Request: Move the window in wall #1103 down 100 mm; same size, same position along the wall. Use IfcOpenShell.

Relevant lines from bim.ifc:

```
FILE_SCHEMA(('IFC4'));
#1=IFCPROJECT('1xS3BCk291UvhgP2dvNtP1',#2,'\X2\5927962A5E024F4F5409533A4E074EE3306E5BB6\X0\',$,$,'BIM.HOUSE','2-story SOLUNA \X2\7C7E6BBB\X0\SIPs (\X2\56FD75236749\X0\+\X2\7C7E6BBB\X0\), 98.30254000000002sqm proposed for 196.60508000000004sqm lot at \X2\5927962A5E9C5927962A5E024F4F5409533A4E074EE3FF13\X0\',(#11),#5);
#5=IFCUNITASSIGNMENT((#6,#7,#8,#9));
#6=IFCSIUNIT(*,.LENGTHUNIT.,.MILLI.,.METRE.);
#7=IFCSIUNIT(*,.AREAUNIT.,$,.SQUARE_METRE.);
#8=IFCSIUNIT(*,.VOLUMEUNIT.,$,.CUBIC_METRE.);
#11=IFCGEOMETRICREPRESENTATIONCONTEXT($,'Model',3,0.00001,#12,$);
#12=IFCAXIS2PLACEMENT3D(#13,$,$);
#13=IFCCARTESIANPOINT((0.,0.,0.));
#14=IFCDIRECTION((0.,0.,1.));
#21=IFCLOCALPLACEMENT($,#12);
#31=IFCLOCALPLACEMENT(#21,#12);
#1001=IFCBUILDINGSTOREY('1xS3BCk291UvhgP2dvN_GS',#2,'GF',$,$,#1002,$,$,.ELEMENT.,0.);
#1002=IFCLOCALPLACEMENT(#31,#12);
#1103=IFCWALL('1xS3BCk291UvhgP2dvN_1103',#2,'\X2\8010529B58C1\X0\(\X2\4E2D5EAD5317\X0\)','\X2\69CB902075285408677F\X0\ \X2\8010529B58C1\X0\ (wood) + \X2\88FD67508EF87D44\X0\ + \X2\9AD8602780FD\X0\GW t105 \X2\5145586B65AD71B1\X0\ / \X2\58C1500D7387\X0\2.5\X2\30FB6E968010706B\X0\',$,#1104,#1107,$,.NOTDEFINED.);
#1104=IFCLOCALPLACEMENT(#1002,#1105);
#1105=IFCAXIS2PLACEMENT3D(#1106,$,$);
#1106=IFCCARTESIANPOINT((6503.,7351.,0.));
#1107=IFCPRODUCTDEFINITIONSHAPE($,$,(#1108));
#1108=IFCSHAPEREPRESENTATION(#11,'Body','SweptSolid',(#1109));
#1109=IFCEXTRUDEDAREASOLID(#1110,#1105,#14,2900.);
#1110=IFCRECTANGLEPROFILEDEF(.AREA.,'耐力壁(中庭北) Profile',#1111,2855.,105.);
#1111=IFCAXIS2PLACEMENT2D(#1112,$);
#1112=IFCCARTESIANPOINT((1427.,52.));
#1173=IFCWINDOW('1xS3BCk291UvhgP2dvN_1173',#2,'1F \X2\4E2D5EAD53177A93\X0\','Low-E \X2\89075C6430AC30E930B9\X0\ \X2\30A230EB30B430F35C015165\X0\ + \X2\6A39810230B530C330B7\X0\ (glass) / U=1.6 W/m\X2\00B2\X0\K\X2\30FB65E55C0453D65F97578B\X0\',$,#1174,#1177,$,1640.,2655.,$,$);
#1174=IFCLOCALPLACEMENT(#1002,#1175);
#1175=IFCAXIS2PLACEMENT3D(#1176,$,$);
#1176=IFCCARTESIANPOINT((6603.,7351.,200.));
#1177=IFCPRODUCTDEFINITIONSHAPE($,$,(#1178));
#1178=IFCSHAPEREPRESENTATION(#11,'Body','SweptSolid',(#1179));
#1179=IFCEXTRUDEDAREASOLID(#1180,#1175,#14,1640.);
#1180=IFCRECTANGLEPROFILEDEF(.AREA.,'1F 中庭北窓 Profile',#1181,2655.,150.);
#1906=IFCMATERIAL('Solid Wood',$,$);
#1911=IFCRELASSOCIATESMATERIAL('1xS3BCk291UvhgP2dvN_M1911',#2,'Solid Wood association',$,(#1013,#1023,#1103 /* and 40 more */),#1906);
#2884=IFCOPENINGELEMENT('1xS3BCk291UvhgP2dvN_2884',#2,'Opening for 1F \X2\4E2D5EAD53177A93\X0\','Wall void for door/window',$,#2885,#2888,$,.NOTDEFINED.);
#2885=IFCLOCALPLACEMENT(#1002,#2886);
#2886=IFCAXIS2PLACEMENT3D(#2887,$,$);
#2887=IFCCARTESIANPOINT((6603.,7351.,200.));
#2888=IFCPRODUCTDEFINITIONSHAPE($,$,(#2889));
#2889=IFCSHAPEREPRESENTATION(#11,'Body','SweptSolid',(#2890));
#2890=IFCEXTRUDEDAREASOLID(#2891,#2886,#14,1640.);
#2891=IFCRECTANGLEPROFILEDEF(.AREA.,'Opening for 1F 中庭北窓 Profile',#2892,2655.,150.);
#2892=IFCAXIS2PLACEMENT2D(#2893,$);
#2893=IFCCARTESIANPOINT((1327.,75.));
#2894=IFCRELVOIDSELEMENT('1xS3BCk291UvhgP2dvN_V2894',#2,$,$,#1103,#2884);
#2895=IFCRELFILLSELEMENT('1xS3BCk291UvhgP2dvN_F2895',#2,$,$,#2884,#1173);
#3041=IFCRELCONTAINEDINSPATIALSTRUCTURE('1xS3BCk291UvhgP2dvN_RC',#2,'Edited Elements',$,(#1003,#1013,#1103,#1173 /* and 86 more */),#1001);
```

```python
import numpy as np
import ifcopenshell
import ifcopenshell.api.geometry
import ifcopenshell.util.placement
import ifcopenshell.util.unit

model = ifcopenshell.open("bim.ifc")
unit_scale = ifcopenshell.util.unit.calculate_unit_scale(model)

window = model.by_guid("1xS3BCk291UvhgP2dvN_1173")
opening = window.FillsVoids[0].RelatingOpeningElement
dz = -100.0

shift = np.array([0.0, 0.0, dz])
# The window is not placed relative to its opening, so move both.
for product in (opening, window):
    matrix = ifcopenshell.util.placement.get_local_placement(product.ObjectPlacement)
    matrix[:3, 3] += shift
    ifcopenshell.api.geometry.edit_object_placement(model, product=product, matrix=matrix, is_si=False)

print(f"moved by {dz * unit_scale:+.3f} m")

model.write("bim_updated.ifc")
```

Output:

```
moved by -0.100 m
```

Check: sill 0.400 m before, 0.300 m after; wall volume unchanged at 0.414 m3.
